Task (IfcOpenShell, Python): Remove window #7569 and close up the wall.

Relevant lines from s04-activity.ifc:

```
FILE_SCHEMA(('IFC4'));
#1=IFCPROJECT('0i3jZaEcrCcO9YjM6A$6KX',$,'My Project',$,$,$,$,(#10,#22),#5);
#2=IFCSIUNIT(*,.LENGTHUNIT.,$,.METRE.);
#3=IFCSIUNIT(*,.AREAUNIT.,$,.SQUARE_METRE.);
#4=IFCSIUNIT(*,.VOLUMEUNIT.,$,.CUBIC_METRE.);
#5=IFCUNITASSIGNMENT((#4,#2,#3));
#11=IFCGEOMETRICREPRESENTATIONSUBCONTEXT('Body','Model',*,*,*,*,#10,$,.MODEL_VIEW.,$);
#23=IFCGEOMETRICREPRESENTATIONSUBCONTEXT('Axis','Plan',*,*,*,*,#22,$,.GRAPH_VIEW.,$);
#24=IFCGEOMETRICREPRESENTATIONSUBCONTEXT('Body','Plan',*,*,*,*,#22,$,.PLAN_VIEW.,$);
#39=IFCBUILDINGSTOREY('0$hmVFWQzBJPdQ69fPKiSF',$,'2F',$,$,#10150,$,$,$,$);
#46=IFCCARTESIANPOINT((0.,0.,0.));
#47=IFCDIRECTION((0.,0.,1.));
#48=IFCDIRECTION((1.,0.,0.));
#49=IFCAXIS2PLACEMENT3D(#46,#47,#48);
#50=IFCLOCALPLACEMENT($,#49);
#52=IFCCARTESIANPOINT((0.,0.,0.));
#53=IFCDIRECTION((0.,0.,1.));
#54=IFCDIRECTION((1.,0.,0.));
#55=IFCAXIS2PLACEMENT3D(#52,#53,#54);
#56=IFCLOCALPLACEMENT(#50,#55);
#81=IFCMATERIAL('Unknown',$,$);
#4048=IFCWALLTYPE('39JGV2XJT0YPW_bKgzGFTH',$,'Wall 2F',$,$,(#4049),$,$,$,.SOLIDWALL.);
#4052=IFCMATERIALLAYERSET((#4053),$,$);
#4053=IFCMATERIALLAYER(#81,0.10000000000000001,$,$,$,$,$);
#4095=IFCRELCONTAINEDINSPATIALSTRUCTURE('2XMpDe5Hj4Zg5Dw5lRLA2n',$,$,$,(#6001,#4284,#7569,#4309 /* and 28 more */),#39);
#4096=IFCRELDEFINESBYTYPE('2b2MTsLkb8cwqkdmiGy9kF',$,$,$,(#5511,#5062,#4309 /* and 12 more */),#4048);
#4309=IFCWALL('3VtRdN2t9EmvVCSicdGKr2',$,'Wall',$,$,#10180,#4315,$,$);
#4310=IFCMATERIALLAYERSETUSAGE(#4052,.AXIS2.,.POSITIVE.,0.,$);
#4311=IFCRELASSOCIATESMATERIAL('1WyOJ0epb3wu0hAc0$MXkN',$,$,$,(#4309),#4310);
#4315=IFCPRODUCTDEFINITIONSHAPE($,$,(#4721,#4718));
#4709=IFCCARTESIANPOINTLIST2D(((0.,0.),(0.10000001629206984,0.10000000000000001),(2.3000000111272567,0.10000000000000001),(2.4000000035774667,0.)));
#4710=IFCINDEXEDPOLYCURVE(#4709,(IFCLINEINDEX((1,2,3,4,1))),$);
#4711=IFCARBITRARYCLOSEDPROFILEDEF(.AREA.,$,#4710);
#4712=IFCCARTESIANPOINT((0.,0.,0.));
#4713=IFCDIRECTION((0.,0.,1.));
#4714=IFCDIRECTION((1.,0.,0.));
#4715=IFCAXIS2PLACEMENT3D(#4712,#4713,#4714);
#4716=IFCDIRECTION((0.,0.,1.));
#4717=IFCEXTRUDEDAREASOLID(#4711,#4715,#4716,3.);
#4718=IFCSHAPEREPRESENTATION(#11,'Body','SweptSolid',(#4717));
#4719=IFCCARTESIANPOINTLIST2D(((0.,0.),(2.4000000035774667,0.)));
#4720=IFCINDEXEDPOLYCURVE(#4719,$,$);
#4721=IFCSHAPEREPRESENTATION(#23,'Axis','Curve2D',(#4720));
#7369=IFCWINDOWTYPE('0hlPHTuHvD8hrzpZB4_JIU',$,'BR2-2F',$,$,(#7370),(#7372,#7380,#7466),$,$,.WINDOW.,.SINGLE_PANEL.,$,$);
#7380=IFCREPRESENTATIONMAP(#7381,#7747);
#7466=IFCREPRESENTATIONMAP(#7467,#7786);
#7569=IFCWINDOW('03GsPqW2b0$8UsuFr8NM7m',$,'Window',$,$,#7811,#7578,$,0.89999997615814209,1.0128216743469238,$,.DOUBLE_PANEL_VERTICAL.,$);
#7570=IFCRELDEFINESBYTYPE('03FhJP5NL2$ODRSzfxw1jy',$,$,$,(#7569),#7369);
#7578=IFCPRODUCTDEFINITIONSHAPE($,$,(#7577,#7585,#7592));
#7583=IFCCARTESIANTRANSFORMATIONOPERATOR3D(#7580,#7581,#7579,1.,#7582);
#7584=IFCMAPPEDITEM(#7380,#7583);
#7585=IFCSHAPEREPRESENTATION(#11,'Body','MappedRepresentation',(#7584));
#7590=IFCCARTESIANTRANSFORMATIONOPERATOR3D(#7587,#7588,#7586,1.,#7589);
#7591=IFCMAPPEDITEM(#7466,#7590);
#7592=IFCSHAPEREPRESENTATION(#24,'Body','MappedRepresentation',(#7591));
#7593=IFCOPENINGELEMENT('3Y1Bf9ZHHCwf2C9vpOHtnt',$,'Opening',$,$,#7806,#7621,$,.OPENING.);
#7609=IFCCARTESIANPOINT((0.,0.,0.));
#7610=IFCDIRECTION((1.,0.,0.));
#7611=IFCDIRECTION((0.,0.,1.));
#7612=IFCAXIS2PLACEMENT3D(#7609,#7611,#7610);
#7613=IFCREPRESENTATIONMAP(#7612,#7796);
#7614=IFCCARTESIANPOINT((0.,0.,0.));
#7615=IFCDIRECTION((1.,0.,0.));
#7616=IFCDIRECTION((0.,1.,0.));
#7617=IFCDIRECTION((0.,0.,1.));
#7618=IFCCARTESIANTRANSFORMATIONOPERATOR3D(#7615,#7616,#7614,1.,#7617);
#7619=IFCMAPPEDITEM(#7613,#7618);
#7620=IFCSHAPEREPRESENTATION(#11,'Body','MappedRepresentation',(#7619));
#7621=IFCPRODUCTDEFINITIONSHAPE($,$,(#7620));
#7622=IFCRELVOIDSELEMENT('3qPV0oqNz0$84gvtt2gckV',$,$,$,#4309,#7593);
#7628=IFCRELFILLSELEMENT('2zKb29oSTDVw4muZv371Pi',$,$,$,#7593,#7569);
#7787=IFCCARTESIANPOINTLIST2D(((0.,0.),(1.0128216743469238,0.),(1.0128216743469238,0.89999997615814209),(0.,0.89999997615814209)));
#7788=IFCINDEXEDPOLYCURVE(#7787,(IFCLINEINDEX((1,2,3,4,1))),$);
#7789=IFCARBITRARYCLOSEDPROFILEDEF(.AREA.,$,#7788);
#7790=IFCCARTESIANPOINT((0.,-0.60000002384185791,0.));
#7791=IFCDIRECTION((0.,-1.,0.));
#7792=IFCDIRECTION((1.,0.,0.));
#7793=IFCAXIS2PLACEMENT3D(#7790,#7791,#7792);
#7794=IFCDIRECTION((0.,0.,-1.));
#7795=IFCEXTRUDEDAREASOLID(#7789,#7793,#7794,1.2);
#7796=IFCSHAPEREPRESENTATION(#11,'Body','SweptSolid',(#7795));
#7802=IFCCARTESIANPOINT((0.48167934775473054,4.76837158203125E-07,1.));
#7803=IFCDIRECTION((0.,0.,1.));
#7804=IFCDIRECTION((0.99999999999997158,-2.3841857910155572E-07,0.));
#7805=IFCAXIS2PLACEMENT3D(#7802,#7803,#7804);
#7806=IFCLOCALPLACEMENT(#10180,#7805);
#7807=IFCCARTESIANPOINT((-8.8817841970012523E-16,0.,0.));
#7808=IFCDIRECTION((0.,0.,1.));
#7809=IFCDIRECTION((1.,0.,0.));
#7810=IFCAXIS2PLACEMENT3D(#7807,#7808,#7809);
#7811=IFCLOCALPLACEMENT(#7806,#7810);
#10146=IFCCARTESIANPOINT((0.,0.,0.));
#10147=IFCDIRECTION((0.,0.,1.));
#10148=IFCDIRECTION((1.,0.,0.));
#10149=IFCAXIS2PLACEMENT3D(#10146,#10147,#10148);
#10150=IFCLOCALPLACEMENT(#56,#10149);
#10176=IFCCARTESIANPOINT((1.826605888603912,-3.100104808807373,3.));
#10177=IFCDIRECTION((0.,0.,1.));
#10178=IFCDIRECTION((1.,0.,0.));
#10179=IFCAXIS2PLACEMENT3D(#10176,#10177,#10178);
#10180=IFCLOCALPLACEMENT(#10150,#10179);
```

```python
import ifcopenshell
import ifcopenshell.api.feature
import ifcopenshell.api.root
import ifcopenshell.geom
import ifcopenshell.util.shape

model = ifcopenshell.open("s04-activity.ifc")
settings = ifcopenshell.geom.settings()


def volume(element):
    """Net volume in cubic metres, openings subtracted."""
    shape = ifcopenshell.geom.create_shape(settings, element)
    return ifcopenshell.util.shape.get_volume(shape.geometry)


window = model.by_guid("03GsPqW2b0$8UsuFr8NM7m")
opening = window.FillsVoids[0].RelatingOpeningElement
wall = opening.VoidsElements[0].RelatingBuildingElement
before = volume(wall)

ifcopenshell.api.root.remove_product(model, product=window)
ifcopenshell.api.feature.remove_feature(model, feature=opening)

after = volume(wall)

print(f"wall volume {before:.3f} -> {after:.3f} m3")

model.write("s04-activity_rev.ifc")
```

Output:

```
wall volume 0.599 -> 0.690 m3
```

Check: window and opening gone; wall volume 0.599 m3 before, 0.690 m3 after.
